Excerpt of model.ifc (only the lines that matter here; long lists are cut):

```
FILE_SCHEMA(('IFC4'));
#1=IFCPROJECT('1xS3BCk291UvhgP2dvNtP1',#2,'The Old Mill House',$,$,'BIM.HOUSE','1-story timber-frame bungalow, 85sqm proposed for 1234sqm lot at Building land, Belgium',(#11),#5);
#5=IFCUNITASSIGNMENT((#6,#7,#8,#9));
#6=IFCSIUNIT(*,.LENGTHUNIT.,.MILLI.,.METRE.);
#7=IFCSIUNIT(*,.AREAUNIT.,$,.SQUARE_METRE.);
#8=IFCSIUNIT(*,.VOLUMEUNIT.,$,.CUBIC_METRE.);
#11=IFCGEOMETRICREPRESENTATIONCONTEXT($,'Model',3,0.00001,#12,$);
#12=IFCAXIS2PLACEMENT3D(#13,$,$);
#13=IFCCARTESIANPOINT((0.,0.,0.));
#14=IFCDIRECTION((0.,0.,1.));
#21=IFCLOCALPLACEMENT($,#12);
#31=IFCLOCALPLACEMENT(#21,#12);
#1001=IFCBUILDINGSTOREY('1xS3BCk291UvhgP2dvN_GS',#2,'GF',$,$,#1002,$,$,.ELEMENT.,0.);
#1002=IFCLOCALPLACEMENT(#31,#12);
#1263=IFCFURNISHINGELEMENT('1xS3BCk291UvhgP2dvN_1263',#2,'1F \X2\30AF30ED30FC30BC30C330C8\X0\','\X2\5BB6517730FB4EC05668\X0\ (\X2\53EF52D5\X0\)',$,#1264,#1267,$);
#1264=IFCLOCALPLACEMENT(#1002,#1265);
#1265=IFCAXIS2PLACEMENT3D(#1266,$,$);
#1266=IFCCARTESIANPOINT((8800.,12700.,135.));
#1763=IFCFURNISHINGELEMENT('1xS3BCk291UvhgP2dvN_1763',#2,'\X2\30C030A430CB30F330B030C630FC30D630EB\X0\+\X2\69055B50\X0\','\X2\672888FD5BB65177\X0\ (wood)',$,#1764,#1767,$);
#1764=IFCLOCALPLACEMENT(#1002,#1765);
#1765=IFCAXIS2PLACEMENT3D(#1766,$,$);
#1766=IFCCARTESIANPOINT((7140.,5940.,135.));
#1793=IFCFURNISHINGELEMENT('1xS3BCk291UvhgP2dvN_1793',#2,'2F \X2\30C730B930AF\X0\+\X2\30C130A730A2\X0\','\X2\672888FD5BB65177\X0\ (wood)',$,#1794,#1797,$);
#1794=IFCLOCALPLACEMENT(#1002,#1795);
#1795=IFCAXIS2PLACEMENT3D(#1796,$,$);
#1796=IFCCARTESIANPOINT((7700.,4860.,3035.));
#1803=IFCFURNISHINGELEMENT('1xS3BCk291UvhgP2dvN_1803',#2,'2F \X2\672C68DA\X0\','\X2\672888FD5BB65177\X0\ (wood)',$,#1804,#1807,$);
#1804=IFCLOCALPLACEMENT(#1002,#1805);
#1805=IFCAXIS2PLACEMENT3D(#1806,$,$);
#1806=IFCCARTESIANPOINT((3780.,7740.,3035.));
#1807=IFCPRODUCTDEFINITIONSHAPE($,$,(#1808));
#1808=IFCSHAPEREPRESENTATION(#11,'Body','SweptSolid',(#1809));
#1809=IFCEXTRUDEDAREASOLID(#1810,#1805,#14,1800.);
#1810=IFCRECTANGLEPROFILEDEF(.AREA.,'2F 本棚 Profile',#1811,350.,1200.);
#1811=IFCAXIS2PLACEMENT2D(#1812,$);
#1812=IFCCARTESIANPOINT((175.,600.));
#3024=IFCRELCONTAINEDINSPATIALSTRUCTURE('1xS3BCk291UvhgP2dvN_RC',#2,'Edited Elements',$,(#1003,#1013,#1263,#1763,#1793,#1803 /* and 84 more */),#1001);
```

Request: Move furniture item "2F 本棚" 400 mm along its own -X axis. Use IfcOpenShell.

```python
import ifcopenshell
import ifcopenshell.api.geometry
import ifcopenshell.util.placement

model = ifcopenshell.open("model.ifc")

item = model.by_guid("1xS3BCk291UvhgP2dvN_1803")
matrix = ifcopenshell.util.placement.get_local_placement(item.ObjectPlacement)
matrix[:3, 3] -= matrix[:3, 0] * 400.0
ifcopenshell.api.geometry.edit_object_placement(model, product=item, matrix=matrix, is_si=False)

print(ifcopenshell.util.placement.get_local_placement(item.ObjectPlacement).round(3) + 0.0)

model.write("model-out.ifc")
```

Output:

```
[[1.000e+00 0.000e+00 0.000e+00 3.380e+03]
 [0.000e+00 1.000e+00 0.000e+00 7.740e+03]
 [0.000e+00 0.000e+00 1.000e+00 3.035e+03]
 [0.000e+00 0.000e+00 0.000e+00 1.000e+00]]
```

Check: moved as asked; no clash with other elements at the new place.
